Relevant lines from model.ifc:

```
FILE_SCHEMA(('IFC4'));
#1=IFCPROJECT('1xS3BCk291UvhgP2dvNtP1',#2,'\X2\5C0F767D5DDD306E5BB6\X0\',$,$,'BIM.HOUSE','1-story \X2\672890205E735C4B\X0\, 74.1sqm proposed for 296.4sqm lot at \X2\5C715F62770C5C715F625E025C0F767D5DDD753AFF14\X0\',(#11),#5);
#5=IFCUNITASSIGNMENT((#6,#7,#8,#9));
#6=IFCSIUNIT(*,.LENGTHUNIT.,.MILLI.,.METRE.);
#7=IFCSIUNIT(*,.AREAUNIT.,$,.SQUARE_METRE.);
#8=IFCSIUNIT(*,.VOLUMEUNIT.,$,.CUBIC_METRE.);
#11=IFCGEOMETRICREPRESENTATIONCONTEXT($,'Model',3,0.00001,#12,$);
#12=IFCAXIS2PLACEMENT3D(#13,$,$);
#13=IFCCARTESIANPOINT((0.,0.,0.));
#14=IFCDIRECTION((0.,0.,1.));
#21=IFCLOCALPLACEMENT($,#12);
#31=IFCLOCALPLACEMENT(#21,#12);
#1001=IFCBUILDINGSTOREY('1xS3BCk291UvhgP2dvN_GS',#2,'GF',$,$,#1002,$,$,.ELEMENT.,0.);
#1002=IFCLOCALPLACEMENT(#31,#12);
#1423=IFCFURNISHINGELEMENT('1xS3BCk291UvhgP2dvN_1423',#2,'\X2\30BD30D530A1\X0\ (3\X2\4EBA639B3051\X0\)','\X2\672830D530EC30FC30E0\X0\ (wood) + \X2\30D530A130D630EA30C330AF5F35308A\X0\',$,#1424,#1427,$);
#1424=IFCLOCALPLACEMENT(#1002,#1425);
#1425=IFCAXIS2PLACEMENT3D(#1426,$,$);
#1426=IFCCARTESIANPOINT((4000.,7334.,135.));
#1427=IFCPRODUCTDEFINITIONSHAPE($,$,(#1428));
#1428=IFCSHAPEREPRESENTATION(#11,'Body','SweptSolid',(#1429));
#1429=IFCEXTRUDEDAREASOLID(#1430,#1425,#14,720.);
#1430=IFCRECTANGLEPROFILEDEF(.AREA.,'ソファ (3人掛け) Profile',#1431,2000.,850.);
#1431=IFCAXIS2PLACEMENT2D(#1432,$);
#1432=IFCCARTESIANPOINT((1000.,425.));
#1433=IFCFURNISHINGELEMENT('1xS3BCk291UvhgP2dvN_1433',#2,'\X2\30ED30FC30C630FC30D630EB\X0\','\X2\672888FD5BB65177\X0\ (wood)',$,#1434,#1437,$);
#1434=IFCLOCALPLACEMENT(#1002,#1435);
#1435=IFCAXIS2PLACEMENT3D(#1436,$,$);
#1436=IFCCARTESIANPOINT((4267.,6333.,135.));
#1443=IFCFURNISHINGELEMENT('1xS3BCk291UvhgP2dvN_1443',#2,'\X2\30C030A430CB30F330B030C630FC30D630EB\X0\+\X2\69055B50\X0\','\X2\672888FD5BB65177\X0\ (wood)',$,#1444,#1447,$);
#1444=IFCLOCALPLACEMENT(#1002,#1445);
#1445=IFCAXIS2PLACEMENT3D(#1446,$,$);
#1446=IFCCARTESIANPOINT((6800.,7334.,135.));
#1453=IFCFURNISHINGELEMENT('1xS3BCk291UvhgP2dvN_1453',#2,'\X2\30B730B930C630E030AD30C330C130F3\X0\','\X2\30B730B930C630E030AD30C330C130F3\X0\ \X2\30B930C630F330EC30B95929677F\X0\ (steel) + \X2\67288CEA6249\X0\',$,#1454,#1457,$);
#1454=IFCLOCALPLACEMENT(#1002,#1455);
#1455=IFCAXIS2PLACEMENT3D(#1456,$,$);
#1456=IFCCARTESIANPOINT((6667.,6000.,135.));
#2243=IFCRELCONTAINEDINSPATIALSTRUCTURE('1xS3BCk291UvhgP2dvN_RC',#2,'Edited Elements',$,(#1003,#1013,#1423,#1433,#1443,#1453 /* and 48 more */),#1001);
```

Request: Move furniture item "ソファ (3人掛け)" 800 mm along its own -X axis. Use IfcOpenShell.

```python
import ifcopenshell
import ifcopenshell.api.geometry
import ifcopenshell.util.placement
import ifcopenshell.util.unit

model = ifcopenshell.open("model.ifc")
unit_scale = ifcopenshell.util.unit.calculate_unit_scale(model)

item = model.by_guid("1xS3BCk291UvhgP2dvN_1423")
matrix = ifcopenshell.util.placement.get_local_placement(item.ObjectPlacement)
matrix[:3, 3] -= matrix[:3, 0] * 0.8 / unit_scale
ifcopenshell.api.geometry.edit_object_placement(model, product=item, matrix=matrix, is_si=False)

print(ifcopenshell.util.placement.get_local_placement(item.ObjectPlacement).round(3) + 0.0)

model.write("model_rev.ifc")
```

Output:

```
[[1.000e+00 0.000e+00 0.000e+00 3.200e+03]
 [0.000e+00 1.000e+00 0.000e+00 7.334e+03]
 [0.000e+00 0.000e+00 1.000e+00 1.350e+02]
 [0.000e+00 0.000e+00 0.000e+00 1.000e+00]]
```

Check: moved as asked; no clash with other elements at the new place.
